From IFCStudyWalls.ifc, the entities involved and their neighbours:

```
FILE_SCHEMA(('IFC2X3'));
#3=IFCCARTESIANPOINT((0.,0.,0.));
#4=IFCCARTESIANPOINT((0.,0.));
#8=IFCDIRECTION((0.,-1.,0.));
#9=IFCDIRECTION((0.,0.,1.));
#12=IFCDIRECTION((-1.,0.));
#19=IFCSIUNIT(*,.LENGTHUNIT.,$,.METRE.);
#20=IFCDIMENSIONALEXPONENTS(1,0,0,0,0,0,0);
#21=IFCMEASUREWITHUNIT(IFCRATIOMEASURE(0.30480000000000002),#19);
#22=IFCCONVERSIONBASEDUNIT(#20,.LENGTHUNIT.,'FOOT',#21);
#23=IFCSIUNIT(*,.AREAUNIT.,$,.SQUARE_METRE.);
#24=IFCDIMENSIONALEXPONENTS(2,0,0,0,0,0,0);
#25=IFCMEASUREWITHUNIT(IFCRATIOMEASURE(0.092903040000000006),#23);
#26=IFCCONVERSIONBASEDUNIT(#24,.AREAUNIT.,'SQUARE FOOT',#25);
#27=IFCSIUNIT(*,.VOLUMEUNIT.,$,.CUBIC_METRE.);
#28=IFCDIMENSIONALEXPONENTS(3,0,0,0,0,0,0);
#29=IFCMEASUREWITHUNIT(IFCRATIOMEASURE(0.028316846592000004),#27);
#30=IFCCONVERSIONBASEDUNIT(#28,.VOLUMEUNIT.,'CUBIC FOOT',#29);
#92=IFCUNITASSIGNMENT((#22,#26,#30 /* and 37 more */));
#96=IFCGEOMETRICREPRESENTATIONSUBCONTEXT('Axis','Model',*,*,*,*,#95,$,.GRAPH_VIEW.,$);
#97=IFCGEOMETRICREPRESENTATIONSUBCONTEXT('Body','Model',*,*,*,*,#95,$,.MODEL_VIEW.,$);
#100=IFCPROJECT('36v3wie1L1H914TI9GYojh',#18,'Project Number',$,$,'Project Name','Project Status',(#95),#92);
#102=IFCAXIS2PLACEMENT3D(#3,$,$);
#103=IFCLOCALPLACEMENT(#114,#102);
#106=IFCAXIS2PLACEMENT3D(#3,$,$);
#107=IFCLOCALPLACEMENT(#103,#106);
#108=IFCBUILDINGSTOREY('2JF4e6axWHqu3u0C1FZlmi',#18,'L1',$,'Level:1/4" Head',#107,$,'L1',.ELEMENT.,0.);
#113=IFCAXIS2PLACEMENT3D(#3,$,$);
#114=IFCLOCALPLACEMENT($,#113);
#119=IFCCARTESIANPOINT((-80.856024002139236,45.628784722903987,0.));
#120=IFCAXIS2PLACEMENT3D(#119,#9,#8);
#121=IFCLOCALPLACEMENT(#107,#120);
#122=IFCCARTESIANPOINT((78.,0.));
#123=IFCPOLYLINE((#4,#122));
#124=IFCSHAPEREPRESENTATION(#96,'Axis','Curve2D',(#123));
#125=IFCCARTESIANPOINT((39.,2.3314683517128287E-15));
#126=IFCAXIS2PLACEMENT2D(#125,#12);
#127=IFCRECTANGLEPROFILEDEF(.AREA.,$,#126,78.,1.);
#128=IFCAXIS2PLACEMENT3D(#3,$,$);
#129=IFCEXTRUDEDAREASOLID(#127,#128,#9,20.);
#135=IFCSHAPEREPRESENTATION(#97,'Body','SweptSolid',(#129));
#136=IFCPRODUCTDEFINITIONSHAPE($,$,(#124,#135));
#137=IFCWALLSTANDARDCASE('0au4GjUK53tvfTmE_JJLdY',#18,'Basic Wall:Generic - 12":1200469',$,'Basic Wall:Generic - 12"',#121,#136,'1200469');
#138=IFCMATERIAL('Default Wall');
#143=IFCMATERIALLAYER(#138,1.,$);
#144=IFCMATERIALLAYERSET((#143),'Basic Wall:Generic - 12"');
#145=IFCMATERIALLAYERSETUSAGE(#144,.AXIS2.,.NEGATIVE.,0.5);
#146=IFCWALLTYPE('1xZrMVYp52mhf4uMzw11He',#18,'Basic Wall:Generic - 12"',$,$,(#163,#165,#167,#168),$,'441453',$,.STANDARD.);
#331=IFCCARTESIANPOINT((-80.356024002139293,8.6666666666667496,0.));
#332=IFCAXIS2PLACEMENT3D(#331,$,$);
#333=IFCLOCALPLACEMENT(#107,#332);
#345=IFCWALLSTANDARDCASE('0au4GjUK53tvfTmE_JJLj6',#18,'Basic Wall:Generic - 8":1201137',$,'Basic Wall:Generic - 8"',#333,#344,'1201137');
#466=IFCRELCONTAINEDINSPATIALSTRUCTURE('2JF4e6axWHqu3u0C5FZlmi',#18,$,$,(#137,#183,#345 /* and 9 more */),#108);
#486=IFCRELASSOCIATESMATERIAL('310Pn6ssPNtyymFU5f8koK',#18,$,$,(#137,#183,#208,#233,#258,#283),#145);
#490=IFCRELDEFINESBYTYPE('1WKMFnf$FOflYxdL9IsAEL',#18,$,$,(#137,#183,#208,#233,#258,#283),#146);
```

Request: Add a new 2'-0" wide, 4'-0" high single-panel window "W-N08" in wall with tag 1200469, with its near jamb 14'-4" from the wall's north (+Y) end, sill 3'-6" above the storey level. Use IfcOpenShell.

```python
import numpy as np
import ifcopenshell
import ifcopenshell.api.feature
import ifcopenshell.api.geometry
import ifcopenshell.api.root
import ifcopenshell.api.spatial
import ifcopenshell.api.type
import ifcopenshell.geom
import ifcopenshell.util.element
import ifcopenshell.util.placement
import ifcopenshell.util.representation
import ifcopenshell.util.shape
import ifcopenshell.util.unit

model = ifcopenshell.open("IFCStudyWalls.ifc")
unit_scale = ifcopenshell.util.unit.calculate_unit_scale(model)
settings = ifcopenshell.geom.settings()


def volume(element):
    """Net volume in cubic metres, openings subtracted."""
    shape = ifcopenshell.geom.create_shape(settings, element)
    return ifcopenshell.util.shape.get_volume(shape.geometry)


wall = model.by_guid("0au4GjUK53tvfTmE_JJLdY")
storey = ifcopenshell.util.element.get_container(wall, ifc_class="IfcBuildingStorey")
context = ifcopenshell.util.representation.get_context(model, "Model", "Body", "MODEL_VIEW")
before = volume(wall)

width, height, from_end, sill = 0.6096, 1.2192, 4.3688, 1.0668  # metres

# The wall runs along its own X axis, and the end named is its -X end.
wall_shape = ifcopenshell.geom.create_shape(settings, wall)
x, y, z = ifcopenshell.util.shape.get_vertices(wall_shape.geometry).T
start = x.min() + from_end
face, thickness = float(y.min()), float(y.max() - y.min())
wall_matrix = ifcopenshell.util.placement.get_local_placement(wall.ObjectPlacement)
level = ifcopenshell.util.placement.get_local_placement(storey.ObjectPlacement)[2, 3]


def in_wall(x, y):
    """Placement at x, y metres in the wall's axes, at sill height."""
    matrix = wall_matrix.copy()
    matrix[:, 3] = wall_matrix @ np.array([x / unit_scale, y / unit_scale, 0.0, 1.0])
    matrix[2, 3] = level + sill / unit_scale
    return matrix


# Opening: a box that overshoots both wall faces by 50 mm.
opening = ifcopenshell.api.root.create_entity(model, ifc_class="IfcOpeningElement")
box = ifcopenshell.api.geometry.add_wall_representation(
    model, context=context, length=width, height=height, thickness=thickness + 0.1
)
ifcopenshell.api.geometry.assign_representation(model, product=opening, representation=box)
ifcopenshell.api.geometry.edit_object_placement(model, product=opening, matrix=in_wall(start, face - 0.05), is_si=False)
ifcopenshell.api.feature.add_feature(model, feature=opening, element=wall)

window = ifcopenshell.api.root.create_entity(model, ifc_class="IfcWindow", name="W-N08")
window.OverallWidth, window.OverallHeight = width / unit_scale, height / unit_scale
body = ifcopenshell.api.geometry.add_window_representation(
    model,
    context=context,
    overall_width=window.OverallWidth,
    overall_height=window.OverallHeight,
    partition_type="SINGLE_PANEL",
)
ifcopenshell.api.geometry.assign_representation(model, product=window, representation=body)
ifcopenshell.api.spatial.assign_container(model, products=[window], relating_structure=storey)
fills = ifcopenshell.api.feature.add_filling(model, opening=opening, element=window)
fills.OwnerHistory = window.OwnerHistory  # required in IFC2X3

# IFC2X3 keeps the operation on the window style.
style = ifcopenshell.api.root.create_entity(model, ifc_class="IfcWindowStyle", name="W-N08")
style.OperationType, style.ConstructionType = "SINGLE_PANEL", "NOTDEFINED"
style.ParameterTakesPrecedence = style.Sizeable = False
ifcopenshell.api.type.assign_type(model, related_objects=[window], relating_type=style)

# Centre the window in the wall's thickness.
ifcopenshell.api.geometry.edit_object_placement(model, product=window, matrix=in_wall(start, face), is_si=False)
window_shape = ifcopenshell.geom.create_shape(settings, window)
depth = ifcopenshell.util.shape.get_vertices(window_shape.geometry)[:, 1]
offset = face + thickness / 2 - (depth.min() + depth.max()) / 2
ifcopenshell.api.geometry.edit_object_placement(model, product=window, matrix=in_wall(start, offset), is_si=False)

after = volume(wall)

print(f"wall volume {before:.3f} -> {after:.3f} m3")

model.write("IFCStudyWalls_rev.ifc")
```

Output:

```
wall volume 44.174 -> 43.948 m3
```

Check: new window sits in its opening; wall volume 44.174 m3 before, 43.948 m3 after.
